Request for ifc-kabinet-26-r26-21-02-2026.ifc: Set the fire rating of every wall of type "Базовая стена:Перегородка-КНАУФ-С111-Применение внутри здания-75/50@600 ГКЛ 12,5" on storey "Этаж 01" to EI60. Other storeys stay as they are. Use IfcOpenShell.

First a look at what the model holds.

```python
import ifcopenshell
import ifcopenshell.util.element

model = ifcopenshell.open("ifc-kabinet-26-r26-21-02-2026.ifc")
print(model.schema)
storey = next(s for s in model.by_type("IfcBuildingStorey") if s.Name == "Этаж 01")
walls = [e for e in ifcopenshell.util.element.get_decomposition(storey) if e.is_a("IfcWall")]
seen = {}
for e in walls:
    element_type = ifcopenshell.util.element.get_type(e)
    key = (element_type.Name if element_type != e and element_type else None, ifcopenshell.util.element.get_pset(e, "Pset_WallCommon", "FireRating"))
    seen[key] = seen.get(key, 0) + 1
for (name, value), count in sorted(seen.items(), key=str):
    print(count, "x", name, "|", value)
```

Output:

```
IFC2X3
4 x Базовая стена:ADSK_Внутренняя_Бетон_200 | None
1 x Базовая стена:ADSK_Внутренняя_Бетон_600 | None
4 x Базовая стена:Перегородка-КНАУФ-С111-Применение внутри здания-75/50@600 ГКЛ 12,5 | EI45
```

```python
import ifcopenshell
import ifcopenshell.api.pset
import ifcopenshell.util.element

model = ifcopenshell.open("ifc-kabinet-26-r26-21-02-2026.ifc")

storey = next(s for s in model.by_type("IfcBuildingStorey") if s.Name == "Этаж 01")
walls = [e for e in ifcopenshell.util.element.get_decomposition(storey) if e.is_a("IfcWall")]

count = 0
for e in walls:
    element_type = ifcopenshell.util.element.get_type(e)
    if element_type in (None, e) or element_type.Name != "Базовая стена:Перегородка-КНАУФ-С111-Применение внутри здания-75/50@600 ГКЛ 12,5":
        continue
    # add_pset returns the element's existing set when there is one.
    pset = ifcopenshell.api.pset.add_pset(model, product=e, name="Pset_WallCommon")
    ifcopenshell.api.pset.edit_pset(model, pset=pset, properties={"FireRating": "EI60"})
    count += 1

print(count, "walls updated")

model.write("ifc-kabinet-26-r26-21-02-2026_rev.ifc")
```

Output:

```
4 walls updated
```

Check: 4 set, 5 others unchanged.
